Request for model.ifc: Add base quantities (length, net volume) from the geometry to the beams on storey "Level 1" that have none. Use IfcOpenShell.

First a look at what the model holds.

```python
import ifcopenshell
import ifcopenshell.util.element
import ifcopenshell.util.unit

model = ifcopenshell.open("model.ifc")
print(model.schema)
for unit_type in ("LENGTHUNIT", "AREAUNIT", "VOLUMEUNIT"):
    print(unit_type, ifcopenshell.util.unit.calculate_unit_scale(model, unit_type))
storey = next(s for s in model.by_type("IfcBuildingStorey") if s.Name == "Level 1")
beams = [e for e in ifcopenshell.util.element.get_decomposition(storey) if e.is_a("IfcBeam")]
for e in sorted(beams, key=lambda e: e.id()):
    print(e.id(), e.is_a(), e.Name, list(ifcopenshell.util.element.get_psets(e, qtos_only=True)), sep=" | ")
```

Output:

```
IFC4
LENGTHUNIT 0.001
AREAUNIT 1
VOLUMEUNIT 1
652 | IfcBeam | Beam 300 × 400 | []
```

```python
import ifcopenshell
import ifcopenshell.api.pset
import ifcopenshell.geom
import ifcopenshell.util.element
import ifcopenshell.util.shape
import ifcopenshell.util.unit

model = ifcopenshell.open("model.ifc")
unit_scale = ifcopenshell.util.unit.calculate_unit_scale(model)
volume_scale = ifcopenshell.util.unit.calculate_unit_scale(model, "VOLUMEUNIT")
settings = ifcopenshell.geom.settings()

storey = next(s for s in model.by_type("IfcBuildingStorey") if s.Name == "Level 1")
beams = [e for e in ifcopenshell.util.element.get_decomposition(storey) if e.is_a("IfcBeam")]

for e in sorted(beams, key=lambda e: e.id()):
    if ifcopenshell.util.element.get_psets(e, qtos_only=True, should_inherit=False):
        continue
    # Geometry comes back in metres, in the element's own axes.
    shape = ifcopenshell.geom.create_shape(settings, e)
    values = {
        "Length": ifcopenshell.util.shape.get_max_xyz(shape.geometry) / unit_scale,
        "NetVolume": ifcopenshell.util.shape.get_volume(shape.geometry) / volume_scale,
    }
    qto = ifcopenshell.api.pset.add_qto(model, product=e, name="Qto_BeamBaseQuantities")
    ifcopenshell.api.pset.edit_qto(model, qto=qto, properties=values)
    print(e.id(), {k: round(v, 3) for k, v in values.items()})

model.write("model-out.ifc")
```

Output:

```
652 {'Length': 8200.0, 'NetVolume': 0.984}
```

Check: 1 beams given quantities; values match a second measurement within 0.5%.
